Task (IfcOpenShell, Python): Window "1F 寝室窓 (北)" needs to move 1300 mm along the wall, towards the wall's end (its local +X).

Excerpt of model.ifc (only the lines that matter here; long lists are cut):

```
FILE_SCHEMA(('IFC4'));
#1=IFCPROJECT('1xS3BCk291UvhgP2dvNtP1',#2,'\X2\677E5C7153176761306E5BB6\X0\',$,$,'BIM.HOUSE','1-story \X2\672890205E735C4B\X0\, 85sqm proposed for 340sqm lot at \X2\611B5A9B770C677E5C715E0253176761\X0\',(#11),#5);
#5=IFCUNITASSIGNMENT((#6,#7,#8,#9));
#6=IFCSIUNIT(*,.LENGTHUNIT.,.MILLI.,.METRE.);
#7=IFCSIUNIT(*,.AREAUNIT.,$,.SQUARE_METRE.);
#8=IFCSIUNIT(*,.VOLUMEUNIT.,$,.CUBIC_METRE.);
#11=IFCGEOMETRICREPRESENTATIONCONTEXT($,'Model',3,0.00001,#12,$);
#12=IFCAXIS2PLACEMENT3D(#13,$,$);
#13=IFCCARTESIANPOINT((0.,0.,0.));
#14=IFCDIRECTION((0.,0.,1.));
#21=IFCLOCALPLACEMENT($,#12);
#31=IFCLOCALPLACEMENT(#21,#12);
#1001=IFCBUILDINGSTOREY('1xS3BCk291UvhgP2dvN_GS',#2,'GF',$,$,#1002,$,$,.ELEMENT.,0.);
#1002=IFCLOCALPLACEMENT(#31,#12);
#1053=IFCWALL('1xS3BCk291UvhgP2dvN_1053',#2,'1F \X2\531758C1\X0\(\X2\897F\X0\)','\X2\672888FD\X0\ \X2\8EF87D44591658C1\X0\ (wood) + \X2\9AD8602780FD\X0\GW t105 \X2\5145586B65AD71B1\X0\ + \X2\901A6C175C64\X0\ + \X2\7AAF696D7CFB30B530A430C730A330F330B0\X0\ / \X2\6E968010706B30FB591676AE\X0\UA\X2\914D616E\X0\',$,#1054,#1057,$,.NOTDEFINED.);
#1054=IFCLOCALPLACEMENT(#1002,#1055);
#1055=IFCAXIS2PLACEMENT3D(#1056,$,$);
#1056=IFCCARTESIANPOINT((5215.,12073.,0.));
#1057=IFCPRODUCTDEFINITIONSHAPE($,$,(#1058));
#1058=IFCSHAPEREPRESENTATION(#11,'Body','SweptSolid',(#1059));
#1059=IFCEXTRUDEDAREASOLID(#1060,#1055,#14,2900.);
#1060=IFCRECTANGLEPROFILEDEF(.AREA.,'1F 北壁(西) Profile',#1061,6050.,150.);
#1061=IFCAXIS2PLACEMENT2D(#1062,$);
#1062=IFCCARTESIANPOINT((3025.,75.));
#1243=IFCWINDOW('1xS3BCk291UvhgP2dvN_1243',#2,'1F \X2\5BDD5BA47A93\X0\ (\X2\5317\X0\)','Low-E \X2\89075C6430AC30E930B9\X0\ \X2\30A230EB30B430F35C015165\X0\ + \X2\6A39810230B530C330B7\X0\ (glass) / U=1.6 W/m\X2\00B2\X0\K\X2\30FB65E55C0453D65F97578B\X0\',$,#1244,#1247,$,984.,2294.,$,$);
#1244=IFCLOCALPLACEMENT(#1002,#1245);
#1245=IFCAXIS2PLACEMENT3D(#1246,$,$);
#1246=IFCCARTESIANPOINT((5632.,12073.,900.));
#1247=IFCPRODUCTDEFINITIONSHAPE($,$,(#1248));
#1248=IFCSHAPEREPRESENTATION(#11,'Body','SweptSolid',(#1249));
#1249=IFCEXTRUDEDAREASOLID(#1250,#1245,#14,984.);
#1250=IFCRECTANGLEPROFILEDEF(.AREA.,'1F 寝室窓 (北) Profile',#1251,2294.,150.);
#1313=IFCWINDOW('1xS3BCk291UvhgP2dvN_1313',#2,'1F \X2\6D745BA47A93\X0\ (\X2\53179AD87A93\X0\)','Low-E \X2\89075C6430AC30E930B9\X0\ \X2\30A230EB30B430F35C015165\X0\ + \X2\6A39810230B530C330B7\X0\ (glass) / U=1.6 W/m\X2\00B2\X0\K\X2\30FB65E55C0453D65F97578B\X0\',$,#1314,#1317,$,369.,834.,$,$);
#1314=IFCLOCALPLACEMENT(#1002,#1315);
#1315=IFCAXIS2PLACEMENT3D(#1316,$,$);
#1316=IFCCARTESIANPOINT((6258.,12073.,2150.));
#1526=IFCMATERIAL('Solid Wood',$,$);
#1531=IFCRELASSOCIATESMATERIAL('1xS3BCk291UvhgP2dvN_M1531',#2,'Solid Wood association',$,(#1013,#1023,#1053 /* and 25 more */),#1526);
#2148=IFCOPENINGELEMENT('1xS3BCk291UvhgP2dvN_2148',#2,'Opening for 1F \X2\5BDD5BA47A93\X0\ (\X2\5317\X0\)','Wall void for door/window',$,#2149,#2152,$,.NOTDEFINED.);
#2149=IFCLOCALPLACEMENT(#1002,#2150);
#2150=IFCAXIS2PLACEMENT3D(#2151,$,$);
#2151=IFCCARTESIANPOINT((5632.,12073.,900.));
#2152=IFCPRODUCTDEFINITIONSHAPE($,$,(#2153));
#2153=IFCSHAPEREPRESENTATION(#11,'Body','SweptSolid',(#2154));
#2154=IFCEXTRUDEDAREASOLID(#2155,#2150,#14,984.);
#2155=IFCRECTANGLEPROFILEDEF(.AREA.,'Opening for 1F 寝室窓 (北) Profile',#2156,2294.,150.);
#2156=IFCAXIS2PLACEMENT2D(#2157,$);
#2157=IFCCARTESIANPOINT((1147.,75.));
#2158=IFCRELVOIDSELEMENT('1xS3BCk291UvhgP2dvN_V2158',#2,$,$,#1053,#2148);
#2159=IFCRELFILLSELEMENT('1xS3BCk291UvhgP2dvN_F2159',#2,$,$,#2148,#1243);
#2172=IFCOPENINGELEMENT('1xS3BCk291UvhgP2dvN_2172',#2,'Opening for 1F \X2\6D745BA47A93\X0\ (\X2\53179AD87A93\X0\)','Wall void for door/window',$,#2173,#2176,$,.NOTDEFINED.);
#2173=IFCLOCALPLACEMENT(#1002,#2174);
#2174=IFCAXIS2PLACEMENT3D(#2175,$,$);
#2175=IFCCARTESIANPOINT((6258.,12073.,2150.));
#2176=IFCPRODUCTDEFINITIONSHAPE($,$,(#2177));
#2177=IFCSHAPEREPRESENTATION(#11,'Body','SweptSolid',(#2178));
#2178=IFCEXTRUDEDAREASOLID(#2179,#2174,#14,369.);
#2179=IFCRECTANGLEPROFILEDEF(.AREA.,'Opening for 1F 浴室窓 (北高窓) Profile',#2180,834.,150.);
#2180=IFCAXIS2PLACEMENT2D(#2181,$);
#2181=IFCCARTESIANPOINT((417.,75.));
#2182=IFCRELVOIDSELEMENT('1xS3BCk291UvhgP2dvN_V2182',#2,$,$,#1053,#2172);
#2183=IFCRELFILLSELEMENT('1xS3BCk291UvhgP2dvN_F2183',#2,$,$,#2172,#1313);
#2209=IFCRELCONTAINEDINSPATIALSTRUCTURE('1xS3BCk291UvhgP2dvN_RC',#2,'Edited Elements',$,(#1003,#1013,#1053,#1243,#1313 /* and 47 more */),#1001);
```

```python
import ifcopenshell
import ifcopenshell.api.geometry
import ifcopenshell.util.placement
import ifcopenshell.util.unit

model = ifcopenshell.open("model.ifc")
unit_scale = ifcopenshell.util.unit.calculate_unit_scale(model)

window = model.by_guid("1xS3BCk291UvhgP2dvN_1243")
opening = window.FillsVoids[0].RelatingOpeningElement
wall = opening.VoidsElements[0].RelatingBuildingElement

wall_matrix = ifcopenshell.util.placement.get_local_placement(wall.ObjectPlacement)
shift = wall_matrix[:3, 0] * 1.3 / unit_scale
before = ifcopenshell.util.placement.get_local_placement(window.ObjectPlacement)[:3, 3].copy()

# The window is not placed relative to its opening, so move both.
for product in (opening, window):
    matrix = ifcopenshell.util.placement.get_local_placement(product.ObjectPlacement)
    matrix[:3, 3] += shift
    ifcopenshell.api.geometry.edit_object_placement(model, product=product, matrix=matrix, is_si=False)

after = ifcopenshell.util.placement.get_local_placement(window.ObjectPlacement)[:3, 3]
print("window moved by", (after - before).round(3) + 0.0)

model.write("model_edited.ifc")
```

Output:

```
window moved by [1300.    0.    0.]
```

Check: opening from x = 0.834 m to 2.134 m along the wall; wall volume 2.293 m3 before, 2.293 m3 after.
